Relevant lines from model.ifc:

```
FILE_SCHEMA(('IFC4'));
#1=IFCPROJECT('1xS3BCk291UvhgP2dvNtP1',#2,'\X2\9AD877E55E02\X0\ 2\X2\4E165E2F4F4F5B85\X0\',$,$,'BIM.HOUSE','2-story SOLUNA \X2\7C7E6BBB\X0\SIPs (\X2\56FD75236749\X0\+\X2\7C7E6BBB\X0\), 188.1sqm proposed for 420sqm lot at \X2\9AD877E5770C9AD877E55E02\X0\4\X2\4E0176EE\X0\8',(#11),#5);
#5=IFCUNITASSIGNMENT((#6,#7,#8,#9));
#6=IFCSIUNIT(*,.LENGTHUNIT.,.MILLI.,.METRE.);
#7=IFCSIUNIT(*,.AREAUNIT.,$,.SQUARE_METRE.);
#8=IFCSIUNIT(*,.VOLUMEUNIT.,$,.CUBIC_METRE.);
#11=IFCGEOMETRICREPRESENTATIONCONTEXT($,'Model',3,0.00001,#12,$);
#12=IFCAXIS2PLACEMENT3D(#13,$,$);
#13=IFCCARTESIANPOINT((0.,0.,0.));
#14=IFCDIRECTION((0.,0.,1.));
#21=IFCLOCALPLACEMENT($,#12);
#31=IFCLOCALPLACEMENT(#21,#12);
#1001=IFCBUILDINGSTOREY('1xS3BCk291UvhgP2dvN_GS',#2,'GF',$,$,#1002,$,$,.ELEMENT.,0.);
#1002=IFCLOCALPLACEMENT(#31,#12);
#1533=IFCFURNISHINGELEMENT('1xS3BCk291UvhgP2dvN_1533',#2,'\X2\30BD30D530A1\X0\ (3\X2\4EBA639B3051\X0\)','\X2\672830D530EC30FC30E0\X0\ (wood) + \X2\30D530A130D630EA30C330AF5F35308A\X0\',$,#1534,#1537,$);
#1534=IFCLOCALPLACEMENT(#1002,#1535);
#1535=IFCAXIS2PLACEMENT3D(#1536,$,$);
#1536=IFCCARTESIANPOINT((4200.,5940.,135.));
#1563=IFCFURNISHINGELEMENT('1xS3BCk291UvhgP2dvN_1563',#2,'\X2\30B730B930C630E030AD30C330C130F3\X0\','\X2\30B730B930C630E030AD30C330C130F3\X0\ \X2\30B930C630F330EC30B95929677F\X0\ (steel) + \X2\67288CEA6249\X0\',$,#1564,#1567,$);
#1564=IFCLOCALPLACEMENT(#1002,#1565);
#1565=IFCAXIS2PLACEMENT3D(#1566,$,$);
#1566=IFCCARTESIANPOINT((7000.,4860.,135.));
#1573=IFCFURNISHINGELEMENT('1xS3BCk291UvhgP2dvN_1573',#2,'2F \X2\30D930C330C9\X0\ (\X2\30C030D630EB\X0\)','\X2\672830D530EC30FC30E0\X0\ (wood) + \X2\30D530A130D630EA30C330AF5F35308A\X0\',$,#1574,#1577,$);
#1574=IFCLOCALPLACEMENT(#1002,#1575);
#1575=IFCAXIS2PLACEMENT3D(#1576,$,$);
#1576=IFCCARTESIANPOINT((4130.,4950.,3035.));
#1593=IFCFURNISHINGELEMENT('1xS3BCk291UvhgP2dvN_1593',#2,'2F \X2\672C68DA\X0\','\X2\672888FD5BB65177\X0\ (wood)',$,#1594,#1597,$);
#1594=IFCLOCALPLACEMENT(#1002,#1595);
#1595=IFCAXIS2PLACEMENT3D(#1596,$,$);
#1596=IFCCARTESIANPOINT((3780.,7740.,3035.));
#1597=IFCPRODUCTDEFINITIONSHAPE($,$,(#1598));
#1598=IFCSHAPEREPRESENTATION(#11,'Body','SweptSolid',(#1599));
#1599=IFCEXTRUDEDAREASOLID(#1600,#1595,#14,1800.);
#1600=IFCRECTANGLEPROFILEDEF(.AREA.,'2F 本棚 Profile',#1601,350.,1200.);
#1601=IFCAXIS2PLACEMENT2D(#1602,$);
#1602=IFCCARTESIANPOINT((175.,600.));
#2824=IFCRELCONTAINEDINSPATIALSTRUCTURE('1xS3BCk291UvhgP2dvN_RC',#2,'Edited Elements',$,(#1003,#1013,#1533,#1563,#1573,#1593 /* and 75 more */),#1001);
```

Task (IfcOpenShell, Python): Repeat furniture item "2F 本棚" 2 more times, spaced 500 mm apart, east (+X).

```python
import numpy as np
import ifcopenshell
import ifcopenshell.api.geometry
import ifcopenshell.api.root
import ifcopenshell.util.element
import ifcopenshell.util.placement
import ifcopenshell.util.unit

model = ifcopenshell.open("model.ifc")
unit_scale = ifcopenshell.util.unit.calculate_unit_scale(model)


def reuse_history(source, copy):
    """copy_class also copies each property set's owner history, people and application; keep the originals."""
    for rel in copy.IsDefinedBy:
        if rel.is_a("IfcRelDefinesByProperties") and (history := rel.RelatingPropertyDefinition.OwnerHistory):
            rel.RelatingPropertyDefinition.OwnerHistory = source.OwnerHistory
            ifcopenshell.util.element.remove_deep2(model, history)


source = model.by_id(1593)
base = ifcopenshell.util.placement.get_local_placement(source.ObjectPlacement)
step = np.array([1.0, 0.0, 0.0]) * 0.5 / unit_scale

for i in range(1, 3):
    copy = ifcopenshell.api.root.copy_class(model, product=source)
    copy.Representation = ifcopenshell.util.element.copy_deep(
        model, source.Representation, exclude=["IfcGeometricRepresentationContext", "IfcRepresentationMap"]
    )
    reuse_history(source, copy)
    matrix = base.copy()
    matrix[:3, 3] += i * step
    print("added at", matrix[:3, 3].round(3) + 0.0)
    ifcopenshell.api.geometry.edit_object_placement(model, product=copy, matrix=matrix, is_si=False)

model.write("model_rev.ifc")
```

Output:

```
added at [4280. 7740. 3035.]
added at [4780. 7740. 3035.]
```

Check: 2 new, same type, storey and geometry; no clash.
